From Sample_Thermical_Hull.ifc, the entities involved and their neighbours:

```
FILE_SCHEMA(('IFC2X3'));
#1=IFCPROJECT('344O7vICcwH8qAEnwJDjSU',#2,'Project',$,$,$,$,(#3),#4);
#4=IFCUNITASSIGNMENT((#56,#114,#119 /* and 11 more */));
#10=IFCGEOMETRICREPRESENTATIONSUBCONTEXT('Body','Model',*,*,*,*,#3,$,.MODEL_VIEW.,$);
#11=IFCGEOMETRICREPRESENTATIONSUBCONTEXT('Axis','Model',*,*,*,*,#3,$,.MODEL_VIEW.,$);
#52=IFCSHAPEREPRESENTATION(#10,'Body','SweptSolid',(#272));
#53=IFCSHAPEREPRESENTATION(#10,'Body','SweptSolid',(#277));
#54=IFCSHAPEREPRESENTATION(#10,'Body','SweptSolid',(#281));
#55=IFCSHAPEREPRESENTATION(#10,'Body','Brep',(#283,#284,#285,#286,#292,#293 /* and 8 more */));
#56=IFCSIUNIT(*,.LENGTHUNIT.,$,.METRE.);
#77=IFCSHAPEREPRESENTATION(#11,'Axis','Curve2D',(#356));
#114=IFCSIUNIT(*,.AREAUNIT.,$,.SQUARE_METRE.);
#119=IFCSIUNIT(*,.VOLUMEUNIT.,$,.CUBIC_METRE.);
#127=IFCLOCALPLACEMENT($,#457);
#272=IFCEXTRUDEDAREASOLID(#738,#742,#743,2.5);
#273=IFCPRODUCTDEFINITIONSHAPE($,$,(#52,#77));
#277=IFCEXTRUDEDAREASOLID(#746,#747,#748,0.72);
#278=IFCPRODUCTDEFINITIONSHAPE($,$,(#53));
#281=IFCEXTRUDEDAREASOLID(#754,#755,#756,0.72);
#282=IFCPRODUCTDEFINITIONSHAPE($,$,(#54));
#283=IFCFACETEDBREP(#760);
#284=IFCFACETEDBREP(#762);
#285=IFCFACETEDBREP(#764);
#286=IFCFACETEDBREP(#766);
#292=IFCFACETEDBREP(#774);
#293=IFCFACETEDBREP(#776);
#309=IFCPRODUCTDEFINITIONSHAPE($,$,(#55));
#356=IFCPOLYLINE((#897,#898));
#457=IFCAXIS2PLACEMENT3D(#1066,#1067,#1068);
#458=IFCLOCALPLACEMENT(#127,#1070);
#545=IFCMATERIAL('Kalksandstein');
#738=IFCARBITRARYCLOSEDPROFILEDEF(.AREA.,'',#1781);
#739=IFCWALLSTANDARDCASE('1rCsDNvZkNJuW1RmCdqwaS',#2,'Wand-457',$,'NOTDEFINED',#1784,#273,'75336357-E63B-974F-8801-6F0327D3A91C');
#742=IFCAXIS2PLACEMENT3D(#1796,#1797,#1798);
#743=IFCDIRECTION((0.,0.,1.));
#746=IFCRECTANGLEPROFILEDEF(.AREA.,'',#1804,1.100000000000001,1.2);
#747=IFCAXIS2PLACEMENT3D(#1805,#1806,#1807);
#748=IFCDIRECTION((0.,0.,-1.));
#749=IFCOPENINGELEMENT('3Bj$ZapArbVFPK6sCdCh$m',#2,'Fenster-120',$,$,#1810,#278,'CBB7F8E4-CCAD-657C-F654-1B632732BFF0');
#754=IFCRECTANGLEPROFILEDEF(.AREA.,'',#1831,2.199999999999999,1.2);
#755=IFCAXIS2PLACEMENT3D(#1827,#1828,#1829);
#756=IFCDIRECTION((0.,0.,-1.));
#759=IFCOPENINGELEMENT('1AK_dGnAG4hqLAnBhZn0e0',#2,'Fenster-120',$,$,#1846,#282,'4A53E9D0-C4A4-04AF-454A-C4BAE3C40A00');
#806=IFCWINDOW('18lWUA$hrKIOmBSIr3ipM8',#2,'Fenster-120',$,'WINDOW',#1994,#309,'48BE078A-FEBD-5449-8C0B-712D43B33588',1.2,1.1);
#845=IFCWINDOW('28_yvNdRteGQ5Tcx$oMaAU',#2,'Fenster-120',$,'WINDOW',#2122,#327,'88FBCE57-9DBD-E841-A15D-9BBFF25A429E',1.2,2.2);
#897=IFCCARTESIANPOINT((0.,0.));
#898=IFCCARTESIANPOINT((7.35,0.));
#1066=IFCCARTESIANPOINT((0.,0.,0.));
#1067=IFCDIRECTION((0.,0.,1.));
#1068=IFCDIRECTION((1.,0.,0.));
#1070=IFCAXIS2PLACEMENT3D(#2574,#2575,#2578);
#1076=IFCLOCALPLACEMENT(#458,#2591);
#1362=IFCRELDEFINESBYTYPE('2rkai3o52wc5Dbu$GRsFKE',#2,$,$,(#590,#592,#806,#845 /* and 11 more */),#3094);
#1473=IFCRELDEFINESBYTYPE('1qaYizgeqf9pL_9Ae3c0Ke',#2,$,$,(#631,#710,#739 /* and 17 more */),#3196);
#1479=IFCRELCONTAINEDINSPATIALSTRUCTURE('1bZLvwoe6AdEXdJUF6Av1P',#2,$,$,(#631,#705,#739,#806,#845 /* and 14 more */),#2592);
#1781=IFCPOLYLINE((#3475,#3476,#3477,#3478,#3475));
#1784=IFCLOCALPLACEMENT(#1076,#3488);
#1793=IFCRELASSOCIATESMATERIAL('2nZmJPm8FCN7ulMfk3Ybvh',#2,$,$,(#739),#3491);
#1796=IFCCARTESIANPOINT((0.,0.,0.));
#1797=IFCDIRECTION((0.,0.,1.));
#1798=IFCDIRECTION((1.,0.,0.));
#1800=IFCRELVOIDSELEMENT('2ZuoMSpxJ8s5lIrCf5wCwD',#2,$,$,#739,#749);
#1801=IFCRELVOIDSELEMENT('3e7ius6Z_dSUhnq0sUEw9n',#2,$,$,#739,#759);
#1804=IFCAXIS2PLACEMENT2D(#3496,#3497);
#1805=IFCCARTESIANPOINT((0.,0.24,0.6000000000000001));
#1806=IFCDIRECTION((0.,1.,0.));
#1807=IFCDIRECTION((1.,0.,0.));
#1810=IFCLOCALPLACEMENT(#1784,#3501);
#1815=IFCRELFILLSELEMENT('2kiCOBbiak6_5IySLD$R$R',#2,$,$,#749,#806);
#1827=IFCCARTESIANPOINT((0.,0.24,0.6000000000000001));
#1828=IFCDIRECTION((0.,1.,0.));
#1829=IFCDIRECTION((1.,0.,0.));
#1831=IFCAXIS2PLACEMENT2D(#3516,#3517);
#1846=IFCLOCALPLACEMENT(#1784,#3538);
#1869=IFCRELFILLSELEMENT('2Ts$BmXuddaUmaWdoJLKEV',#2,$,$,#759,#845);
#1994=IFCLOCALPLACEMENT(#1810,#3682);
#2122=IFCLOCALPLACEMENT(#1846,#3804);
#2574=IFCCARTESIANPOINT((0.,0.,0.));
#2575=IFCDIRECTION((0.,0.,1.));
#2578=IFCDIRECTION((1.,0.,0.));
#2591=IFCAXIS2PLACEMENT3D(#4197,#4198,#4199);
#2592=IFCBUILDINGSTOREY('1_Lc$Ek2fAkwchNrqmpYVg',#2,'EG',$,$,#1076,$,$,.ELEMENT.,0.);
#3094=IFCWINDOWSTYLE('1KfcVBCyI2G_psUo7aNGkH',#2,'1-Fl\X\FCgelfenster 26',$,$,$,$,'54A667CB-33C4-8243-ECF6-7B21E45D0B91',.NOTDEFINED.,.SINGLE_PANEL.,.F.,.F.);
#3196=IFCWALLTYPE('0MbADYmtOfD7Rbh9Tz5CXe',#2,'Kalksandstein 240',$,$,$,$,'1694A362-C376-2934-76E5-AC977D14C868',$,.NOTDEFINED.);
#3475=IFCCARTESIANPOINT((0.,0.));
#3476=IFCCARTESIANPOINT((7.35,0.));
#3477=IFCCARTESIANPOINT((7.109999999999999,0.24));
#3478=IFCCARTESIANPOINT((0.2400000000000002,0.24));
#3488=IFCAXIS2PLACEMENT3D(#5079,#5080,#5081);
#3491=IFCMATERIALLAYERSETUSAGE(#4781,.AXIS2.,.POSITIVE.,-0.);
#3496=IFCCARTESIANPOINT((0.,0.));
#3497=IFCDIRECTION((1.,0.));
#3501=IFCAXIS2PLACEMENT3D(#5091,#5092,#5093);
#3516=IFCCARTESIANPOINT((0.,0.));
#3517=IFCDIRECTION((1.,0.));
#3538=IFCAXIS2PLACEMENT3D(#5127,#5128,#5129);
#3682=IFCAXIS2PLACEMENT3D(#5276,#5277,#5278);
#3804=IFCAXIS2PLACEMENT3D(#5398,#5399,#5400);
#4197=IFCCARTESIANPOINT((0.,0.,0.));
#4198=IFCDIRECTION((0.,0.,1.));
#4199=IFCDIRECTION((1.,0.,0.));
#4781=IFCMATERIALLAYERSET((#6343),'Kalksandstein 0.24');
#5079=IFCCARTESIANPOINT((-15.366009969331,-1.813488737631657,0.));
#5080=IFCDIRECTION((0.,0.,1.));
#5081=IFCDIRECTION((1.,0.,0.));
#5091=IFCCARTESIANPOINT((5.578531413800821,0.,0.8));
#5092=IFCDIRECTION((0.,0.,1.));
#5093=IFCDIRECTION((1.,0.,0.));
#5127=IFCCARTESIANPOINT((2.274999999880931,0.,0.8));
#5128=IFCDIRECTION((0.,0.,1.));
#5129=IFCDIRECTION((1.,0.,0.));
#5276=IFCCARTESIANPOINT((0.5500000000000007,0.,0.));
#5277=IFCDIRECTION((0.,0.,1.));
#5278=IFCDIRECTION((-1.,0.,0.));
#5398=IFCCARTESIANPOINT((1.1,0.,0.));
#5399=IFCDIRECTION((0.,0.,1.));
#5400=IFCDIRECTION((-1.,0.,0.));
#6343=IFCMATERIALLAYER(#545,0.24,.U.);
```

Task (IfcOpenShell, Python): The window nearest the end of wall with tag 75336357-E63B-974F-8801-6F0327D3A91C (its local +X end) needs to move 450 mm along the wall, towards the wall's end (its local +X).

```python
import ifcopenshell
import ifcopenshell.api.geometry
import ifcopenshell.util.placement
import ifcopenshell.util.unit

model = ifcopenshell.open("Sample_Thermical_Hull.ifc")
unit_scale = ifcopenshell.util.unit.calculate_unit_scale(model)

window = model.by_guid("18lWUA$hrKIOmBSIr3ipM8")
opening = window.FillsVoids[0].RelatingOpeningElement
wall = opening.VoidsElements[0].RelatingBuildingElement

wall_matrix = ifcopenshell.util.placement.get_local_placement(wall.ObjectPlacement)
shift = wall_matrix[:3, 0] * 0.45 / unit_scale
before = ifcopenshell.util.placement.get_local_placement(window.ObjectPlacement)[:3, 3].copy()

# The window is placed relative to its opening, so it follows when the opening moves.
matrix = ifcopenshell.util.placement.get_local_placement(opening.ObjectPlacement)
matrix[:3, 3] += shift
ifcopenshell.api.geometry.edit_object_placement(
    model, product=opening, matrix=matrix, is_si=False, should_transform_children=True
)

after = ifcopenshell.util.placement.get_local_placement(window.ObjectPlacement)[:3, 3]
print("window moved by", (after - before).round(3) + 0.0)

model.write("Sample_Thermical_Hull_v2.ifc")
```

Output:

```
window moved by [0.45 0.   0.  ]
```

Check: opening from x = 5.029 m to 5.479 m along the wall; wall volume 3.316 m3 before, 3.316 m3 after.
